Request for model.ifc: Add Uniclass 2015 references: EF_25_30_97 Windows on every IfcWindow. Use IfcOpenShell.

First a look at what the model holds.

```python
import ifcopenshell

model = ifcopenshell.open("model.ifc")
print(model.schema)
print("classifications:", [c.Name for c in model.by_type("IfcClassification")])
for ifc_class in ("IfcDoor", "IfcRoof", "IfcStair", "IfcWall", "IfcWindow"):
    print(ifc_class, len(model.by_type(ifc_class)))
```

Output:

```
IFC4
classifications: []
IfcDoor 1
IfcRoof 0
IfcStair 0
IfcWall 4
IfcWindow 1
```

```python
import ifcopenshell
import ifcopenshell.api.classification

model = ifcopenshell.open("model.ifc")

system = ifcopenshell.api.classification.add_classification(model, classification="Uniclass 2015")

codes = {
    "IfcWindow": ("EF_25_30_97", "Windows"),
}
for ifc_class, (code, name) in codes.items():
    products = model.by_type(ifc_class)
    ifcopenshell.api.classification.add_reference(
        model, products=products, classification=system, identification=code, name=name
    )
    print(code, len(products))

model.write("model-out.ifc")
```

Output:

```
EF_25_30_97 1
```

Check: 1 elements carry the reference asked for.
